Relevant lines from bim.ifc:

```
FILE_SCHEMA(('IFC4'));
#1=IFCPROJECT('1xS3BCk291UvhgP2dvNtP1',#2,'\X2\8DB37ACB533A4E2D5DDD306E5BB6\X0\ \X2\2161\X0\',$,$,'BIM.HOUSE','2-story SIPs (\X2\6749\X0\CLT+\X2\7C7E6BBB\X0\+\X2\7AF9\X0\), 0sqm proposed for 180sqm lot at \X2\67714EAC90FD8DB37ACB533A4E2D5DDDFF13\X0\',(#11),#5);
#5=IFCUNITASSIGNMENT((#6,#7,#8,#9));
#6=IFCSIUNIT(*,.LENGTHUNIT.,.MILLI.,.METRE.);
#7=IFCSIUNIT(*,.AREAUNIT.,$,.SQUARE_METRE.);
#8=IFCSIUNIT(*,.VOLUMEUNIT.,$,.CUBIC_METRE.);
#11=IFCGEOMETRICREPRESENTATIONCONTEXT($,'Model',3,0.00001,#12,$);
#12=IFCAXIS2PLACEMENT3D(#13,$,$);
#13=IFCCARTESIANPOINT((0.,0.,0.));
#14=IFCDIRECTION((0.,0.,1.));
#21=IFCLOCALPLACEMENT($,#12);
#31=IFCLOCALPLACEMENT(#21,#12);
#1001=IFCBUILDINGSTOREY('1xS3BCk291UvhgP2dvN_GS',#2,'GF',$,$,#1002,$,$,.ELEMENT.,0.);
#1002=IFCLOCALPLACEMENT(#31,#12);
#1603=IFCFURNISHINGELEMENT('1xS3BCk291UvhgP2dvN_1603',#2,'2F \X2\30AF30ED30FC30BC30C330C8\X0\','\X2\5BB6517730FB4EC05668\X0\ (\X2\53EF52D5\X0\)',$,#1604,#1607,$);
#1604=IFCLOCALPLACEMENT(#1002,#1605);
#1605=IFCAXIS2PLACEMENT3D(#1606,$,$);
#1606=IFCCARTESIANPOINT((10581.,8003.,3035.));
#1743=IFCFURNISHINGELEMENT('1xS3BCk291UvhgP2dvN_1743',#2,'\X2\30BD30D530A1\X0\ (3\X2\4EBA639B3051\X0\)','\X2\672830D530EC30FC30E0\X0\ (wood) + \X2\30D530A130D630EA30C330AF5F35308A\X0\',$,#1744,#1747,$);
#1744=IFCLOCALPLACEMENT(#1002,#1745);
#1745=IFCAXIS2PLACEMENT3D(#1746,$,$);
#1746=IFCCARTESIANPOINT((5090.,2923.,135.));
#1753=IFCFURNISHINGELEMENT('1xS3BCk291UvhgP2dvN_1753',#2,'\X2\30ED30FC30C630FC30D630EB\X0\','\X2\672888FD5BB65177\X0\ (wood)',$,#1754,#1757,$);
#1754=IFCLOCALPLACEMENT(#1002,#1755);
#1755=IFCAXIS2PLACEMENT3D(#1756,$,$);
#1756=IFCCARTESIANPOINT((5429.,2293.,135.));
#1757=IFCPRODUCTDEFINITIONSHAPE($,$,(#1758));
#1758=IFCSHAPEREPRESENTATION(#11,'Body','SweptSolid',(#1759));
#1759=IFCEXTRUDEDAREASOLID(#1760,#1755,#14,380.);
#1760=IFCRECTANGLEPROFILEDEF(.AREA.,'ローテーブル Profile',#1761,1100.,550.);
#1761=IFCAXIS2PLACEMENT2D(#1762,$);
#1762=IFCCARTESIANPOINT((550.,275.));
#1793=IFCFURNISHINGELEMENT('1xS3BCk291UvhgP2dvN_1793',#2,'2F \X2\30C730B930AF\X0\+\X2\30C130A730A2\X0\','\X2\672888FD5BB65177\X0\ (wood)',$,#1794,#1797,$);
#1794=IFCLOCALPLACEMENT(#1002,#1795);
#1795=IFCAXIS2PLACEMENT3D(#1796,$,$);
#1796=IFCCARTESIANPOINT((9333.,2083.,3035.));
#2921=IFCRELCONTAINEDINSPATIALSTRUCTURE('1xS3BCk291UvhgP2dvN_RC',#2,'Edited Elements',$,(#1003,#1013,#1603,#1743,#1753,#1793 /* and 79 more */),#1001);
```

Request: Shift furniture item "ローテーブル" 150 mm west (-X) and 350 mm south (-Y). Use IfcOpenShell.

```python
import ifcopenshell
import ifcopenshell.api.geometry
import ifcopenshell.util.placement

model = ifcopenshell.open("bim.ifc")

item = model.by_guid("1xS3BCk291UvhgP2dvN_1753")
matrix = ifcopenshell.util.placement.get_local_placement(item.ObjectPlacement)
matrix[0, 3] -= 150.0
matrix[1, 3] -= 350.0
ifcopenshell.api.geometry.edit_object_placement(model, product=item, matrix=matrix, is_si=False)

print(ifcopenshell.util.placement.get_local_placement(item.ObjectPlacement).round(3) + 0.0)

model.write("bim_v2.ifc")
```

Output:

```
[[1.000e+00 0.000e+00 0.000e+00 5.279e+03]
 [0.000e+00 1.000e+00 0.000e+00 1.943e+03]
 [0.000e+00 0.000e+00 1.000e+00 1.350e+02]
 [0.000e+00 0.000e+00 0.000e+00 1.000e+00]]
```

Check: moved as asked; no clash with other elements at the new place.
